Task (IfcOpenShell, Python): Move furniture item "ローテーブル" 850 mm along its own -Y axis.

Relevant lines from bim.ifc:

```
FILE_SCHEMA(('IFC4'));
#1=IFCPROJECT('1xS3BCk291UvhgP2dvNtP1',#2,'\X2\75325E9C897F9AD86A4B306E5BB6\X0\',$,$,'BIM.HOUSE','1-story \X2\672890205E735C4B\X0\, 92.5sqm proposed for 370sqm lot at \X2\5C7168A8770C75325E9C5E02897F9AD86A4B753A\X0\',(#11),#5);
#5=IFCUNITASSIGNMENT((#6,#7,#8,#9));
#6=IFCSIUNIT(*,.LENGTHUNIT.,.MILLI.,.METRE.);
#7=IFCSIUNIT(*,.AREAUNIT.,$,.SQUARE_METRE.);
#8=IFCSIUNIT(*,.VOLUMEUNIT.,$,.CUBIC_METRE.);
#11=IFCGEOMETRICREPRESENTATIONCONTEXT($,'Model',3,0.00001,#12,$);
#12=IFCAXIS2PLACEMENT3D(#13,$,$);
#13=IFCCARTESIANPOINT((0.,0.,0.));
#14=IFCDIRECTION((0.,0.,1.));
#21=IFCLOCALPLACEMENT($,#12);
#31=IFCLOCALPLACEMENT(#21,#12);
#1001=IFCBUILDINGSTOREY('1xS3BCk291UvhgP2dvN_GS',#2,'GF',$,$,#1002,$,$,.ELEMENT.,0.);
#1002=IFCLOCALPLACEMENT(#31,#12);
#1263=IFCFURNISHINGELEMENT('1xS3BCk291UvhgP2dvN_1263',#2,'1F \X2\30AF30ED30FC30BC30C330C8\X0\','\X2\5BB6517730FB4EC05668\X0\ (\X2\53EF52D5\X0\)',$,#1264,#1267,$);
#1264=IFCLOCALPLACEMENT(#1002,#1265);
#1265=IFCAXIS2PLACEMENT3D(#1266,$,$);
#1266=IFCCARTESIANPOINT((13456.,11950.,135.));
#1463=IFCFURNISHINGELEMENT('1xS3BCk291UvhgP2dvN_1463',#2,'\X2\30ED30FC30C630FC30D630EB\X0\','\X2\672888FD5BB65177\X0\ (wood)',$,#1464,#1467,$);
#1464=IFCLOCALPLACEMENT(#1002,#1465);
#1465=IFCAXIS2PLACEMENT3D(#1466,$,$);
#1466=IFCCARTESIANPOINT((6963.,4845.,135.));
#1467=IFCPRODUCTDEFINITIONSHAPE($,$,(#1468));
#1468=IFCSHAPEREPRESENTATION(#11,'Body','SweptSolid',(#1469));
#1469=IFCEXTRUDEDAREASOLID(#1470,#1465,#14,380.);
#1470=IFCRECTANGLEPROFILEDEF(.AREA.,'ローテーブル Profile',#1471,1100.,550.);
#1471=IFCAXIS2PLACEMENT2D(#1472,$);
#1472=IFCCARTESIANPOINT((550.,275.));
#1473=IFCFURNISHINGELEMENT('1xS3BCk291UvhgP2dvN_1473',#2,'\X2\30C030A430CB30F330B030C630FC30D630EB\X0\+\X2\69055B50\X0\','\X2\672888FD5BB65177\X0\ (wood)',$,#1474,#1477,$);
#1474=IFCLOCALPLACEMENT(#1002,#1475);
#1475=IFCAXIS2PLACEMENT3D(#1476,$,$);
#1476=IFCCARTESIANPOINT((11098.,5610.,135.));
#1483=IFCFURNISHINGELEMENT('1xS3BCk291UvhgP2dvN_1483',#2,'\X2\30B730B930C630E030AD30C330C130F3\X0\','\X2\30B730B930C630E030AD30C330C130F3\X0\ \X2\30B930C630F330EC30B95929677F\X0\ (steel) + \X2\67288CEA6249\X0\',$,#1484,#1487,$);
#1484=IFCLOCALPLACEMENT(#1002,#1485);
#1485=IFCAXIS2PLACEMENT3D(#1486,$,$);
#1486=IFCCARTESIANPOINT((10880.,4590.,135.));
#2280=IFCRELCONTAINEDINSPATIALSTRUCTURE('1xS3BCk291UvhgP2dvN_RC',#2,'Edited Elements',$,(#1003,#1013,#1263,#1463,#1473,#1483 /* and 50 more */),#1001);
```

```python
import ifcopenshell
import ifcopenshell.api.geometry
import ifcopenshell.util.placement
import ifcopenshell.util.unit

model = ifcopenshell.open("bim.ifc")
unit_scale = ifcopenshell.util.unit.calculate_unit_scale(model)

item = model.by_id(1463)
matrix = ifcopenshell.util.placement.get_local_placement(item.ObjectPlacement)
matrix[:3, 3] -= matrix[:3, 1] * 0.85 / unit_scale
ifcopenshell.api.geometry.edit_object_placement(model, product=item, matrix=matrix, is_si=False)

print(ifcopenshell.util.placement.get_local_placement(item.ObjectPlacement).round(3) + 0.0)

model.write("bim-out.ifc")
```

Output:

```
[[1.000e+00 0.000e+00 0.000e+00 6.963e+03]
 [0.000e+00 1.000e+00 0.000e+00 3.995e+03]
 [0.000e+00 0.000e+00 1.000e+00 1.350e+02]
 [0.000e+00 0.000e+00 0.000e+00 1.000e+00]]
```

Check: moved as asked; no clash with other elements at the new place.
